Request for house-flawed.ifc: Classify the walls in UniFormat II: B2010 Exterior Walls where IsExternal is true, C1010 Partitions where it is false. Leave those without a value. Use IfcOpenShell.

First a look at what the model holds.

```python
import ifcopenshell
import ifcopenshell.util.element

model = ifcopenshell.open("house-flawed.ifc")
print(model.schema)
print("classifications:", [c.Name for c in model.by_type("IfcClassification")])
values = [ifcopenshell.util.element.get_pset(e, "Pset_WallCommon", "IsExternal") for e in model.by_type("IfcWall")]
for value in (True, False, None):
    print("IsExternal", value, values.count(value))
```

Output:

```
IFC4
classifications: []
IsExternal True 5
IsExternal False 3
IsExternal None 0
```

```python
import ifcopenshell
import ifcopenshell.api.classification
import ifcopenshell.util.element

model = ifcopenshell.open("house-flawed.ifc")

system = ifcopenshell.api.classification.add_classification(model, classification="UniFormat II")

walls = model.by_type("IfcWall")
external = {e: ifcopenshell.util.element.get_pset(e, "Pset_WallCommon", "IsExternal") for e in walls}
for flag, code, name in ((True, "B2010", "Exterior Walls"), (False, "C1010", "Partitions")):
    products = [e for e in walls if external[e] is flag]
    ifcopenshell.api.classification.add_reference(
        model, products=products, classification=system, identification=code, name=name
    )
    print(code, len(products))

model.write("house-flawed_v2.ifc")
```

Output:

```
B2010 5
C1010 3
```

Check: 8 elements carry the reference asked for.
